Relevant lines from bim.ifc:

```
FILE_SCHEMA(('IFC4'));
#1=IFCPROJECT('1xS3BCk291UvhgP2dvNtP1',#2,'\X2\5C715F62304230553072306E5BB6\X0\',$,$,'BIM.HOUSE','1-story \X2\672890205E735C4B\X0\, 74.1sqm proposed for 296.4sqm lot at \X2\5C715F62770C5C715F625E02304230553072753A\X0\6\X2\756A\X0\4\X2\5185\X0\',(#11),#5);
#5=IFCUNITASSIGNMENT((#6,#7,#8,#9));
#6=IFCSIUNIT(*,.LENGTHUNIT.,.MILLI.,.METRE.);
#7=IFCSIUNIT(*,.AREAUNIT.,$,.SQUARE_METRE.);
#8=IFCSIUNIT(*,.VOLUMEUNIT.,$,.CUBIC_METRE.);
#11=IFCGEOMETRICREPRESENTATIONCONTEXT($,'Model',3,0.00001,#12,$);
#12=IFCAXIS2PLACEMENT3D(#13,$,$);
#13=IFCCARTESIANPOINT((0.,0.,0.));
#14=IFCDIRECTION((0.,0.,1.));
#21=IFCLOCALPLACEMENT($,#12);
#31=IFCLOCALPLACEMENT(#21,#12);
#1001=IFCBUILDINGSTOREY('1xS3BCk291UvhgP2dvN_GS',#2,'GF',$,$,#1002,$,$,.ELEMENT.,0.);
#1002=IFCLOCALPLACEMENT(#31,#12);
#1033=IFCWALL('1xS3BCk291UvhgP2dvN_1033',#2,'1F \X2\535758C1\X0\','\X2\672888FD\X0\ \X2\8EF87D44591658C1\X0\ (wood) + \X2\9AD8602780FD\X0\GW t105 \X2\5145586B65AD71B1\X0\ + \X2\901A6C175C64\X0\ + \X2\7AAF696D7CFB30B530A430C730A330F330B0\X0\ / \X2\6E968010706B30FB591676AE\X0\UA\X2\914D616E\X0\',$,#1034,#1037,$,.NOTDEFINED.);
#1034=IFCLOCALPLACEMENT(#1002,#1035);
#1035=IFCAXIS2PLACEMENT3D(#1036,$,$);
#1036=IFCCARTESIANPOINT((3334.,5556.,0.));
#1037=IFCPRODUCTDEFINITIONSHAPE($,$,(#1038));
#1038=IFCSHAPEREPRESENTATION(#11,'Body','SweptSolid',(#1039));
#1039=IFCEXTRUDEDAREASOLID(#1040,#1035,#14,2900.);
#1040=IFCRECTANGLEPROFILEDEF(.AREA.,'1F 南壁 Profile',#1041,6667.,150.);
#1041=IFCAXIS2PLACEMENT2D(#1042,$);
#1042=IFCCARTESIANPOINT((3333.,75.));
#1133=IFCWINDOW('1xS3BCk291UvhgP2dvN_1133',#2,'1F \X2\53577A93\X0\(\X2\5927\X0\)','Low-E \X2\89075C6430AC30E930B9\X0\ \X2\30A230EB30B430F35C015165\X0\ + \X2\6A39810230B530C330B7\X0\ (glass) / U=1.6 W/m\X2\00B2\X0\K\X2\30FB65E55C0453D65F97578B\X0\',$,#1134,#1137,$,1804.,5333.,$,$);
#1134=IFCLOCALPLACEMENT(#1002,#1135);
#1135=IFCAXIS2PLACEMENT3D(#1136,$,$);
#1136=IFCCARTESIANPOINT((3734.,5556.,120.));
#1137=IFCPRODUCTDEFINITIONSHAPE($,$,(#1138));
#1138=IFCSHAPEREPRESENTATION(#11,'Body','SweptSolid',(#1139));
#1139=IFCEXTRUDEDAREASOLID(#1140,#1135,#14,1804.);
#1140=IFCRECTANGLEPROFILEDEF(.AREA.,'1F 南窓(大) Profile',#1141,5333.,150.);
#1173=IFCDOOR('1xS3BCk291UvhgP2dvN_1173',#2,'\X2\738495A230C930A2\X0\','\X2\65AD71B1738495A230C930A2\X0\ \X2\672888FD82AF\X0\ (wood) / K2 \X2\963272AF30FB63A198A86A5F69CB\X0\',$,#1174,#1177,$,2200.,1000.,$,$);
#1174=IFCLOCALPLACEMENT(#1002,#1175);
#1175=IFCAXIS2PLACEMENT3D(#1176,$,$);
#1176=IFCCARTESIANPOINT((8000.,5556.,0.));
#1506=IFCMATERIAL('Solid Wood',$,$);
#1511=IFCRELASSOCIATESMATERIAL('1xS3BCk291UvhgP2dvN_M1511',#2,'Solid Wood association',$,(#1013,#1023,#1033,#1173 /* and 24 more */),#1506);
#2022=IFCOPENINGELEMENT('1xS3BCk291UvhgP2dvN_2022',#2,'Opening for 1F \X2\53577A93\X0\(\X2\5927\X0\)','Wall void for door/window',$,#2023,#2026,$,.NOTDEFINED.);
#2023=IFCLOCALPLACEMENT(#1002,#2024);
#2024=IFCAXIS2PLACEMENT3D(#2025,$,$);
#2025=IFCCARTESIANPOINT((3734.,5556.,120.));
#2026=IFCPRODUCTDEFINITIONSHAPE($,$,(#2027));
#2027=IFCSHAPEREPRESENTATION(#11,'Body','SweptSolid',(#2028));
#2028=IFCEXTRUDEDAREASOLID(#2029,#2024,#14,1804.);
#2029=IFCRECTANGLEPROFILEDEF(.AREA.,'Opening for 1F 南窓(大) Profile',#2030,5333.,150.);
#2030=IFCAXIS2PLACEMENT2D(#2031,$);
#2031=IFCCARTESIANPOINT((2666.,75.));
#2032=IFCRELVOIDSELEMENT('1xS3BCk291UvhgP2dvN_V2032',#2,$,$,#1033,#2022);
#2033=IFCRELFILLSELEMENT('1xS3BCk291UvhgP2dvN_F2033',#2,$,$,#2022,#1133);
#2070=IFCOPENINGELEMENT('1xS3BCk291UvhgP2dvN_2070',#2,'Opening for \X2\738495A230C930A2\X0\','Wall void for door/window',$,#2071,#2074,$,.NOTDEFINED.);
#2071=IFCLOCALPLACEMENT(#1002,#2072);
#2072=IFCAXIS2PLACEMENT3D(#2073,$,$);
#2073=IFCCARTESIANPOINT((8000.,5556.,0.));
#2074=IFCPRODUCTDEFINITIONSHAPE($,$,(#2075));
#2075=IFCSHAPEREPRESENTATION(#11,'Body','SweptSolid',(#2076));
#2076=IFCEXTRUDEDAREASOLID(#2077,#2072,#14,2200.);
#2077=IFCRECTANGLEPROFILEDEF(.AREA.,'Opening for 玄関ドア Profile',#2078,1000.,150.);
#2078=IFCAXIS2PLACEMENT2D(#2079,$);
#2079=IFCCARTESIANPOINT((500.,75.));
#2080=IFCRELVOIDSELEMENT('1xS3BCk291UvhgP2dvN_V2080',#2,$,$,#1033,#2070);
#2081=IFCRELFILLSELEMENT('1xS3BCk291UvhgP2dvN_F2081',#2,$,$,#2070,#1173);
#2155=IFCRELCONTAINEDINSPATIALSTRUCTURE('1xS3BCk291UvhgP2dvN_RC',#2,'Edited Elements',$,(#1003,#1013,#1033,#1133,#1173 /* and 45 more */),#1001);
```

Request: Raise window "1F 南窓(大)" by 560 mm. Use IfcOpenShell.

```python
import numpy as np
import ifcopenshell
import ifcopenshell.api.geometry
import ifcopenshell.util.placement
import ifcopenshell.util.unit

model = ifcopenshell.open("bim.ifc")
unit_scale = ifcopenshell.util.unit.calculate_unit_scale(model)

window = model.by_id(1133)
opening = window.FillsVoids[0].RelatingOpeningElement
dz = 560.0

shift = np.array([0.0, 0.0, dz])
# The window is not placed relative to its opening, so move both.
for product in (opening, window):
    matrix = ifcopenshell.util.placement.get_local_placement(product.ObjectPlacement)
    matrix[:3, 3] += shift
    ifcopenshell.api.geometry.edit_object_placement(model, product=product, matrix=matrix, is_si=False)

print(f"moved by {dz * unit_scale:+.3f} m")

model.write("bim-out.ifc")
```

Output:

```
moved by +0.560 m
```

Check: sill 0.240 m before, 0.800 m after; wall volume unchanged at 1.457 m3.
